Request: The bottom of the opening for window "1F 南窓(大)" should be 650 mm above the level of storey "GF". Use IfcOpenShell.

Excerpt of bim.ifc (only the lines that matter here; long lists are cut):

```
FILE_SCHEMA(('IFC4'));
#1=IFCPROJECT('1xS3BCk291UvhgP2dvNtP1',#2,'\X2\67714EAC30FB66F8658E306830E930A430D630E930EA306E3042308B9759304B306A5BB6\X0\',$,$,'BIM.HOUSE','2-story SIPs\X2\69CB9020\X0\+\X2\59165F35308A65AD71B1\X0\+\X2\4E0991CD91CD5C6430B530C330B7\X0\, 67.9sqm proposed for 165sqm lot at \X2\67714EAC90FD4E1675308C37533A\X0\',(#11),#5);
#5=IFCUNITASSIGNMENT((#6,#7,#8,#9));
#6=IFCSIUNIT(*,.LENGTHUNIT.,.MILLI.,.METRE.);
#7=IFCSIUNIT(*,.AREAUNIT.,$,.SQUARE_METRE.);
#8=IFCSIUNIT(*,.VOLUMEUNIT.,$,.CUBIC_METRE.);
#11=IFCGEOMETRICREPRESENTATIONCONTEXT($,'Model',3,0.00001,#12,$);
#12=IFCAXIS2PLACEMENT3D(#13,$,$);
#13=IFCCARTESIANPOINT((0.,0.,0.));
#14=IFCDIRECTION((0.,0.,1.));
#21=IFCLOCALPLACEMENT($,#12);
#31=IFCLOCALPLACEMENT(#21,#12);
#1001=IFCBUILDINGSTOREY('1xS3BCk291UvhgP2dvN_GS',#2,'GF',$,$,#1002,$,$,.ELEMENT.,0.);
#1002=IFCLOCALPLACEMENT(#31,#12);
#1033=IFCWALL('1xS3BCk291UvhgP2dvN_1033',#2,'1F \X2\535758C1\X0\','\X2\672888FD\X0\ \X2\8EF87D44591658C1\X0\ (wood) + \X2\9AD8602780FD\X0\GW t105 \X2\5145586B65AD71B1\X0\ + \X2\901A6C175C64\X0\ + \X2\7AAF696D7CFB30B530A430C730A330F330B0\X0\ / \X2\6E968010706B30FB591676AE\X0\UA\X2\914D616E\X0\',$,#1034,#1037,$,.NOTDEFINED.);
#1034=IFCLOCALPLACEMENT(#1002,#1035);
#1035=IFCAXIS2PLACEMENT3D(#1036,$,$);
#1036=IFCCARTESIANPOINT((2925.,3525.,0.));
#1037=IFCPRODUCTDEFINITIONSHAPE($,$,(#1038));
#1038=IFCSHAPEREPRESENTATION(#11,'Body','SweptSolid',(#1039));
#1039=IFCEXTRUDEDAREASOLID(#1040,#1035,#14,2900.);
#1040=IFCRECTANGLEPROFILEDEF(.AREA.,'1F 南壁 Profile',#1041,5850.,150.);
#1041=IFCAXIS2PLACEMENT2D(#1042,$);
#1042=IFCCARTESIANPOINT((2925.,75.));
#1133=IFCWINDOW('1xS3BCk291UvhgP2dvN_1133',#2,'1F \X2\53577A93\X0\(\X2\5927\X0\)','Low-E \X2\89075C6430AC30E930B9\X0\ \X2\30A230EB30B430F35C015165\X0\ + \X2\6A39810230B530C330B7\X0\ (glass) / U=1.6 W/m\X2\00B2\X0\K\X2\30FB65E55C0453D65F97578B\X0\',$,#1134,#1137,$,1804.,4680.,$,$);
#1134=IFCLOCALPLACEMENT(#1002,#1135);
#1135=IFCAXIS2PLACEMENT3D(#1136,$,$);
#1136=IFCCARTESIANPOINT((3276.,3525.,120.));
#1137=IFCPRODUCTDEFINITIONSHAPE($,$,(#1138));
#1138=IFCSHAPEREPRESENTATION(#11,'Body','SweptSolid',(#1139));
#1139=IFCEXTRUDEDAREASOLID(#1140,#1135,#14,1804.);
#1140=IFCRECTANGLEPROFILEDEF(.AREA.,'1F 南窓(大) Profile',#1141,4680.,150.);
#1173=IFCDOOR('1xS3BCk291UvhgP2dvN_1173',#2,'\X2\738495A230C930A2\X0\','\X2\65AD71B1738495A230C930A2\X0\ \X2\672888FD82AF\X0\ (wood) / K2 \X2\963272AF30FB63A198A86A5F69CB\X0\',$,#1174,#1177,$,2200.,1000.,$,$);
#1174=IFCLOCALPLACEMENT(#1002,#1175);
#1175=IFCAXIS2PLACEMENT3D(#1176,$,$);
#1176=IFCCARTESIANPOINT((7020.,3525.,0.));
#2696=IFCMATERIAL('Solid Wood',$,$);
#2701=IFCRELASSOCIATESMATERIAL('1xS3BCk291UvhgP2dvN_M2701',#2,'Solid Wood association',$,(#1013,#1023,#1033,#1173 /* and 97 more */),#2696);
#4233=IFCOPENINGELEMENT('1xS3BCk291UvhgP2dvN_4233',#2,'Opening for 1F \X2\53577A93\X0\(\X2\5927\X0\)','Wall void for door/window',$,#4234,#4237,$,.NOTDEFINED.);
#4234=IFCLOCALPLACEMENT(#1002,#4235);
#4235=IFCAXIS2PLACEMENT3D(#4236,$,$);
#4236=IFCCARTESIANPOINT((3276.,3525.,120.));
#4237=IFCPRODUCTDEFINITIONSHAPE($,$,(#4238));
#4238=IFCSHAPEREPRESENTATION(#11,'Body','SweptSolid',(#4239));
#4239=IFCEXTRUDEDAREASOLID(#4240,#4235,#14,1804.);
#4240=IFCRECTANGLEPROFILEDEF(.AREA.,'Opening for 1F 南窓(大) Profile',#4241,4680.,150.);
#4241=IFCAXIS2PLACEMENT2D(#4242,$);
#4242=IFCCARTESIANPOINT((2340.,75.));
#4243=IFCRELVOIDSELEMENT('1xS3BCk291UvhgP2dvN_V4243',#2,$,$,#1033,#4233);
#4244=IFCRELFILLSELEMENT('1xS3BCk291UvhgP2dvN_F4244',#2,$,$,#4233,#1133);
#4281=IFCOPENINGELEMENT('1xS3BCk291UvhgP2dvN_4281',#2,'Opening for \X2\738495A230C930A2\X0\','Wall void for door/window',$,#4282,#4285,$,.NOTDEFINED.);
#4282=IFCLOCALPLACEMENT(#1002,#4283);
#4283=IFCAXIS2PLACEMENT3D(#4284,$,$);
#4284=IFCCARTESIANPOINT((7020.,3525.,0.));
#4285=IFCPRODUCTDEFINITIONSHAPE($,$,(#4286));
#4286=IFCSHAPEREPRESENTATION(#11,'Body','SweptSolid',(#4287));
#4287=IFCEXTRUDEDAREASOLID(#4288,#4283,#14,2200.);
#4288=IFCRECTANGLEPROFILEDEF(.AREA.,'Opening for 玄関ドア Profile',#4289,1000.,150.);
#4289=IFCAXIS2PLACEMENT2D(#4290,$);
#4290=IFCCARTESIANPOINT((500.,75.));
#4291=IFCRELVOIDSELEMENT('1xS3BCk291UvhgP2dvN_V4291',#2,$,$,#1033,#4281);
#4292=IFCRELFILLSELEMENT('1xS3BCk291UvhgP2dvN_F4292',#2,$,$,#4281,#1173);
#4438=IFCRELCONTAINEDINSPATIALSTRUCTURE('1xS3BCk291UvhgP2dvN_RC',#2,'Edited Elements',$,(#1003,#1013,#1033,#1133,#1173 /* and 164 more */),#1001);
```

```python
import numpy as np
import ifcopenshell
import ifcopenshell.api.geometry
import ifcopenshell.geom
import ifcopenshell.util.element
import ifcopenshell.util.placement
import ifcopenshell.util.shape
import ifcopenshell.util.unit

model = ifcopenshell.open("bim.ifc")
unit_scale = ifcopenshell.util.unit.calculate_unit_scale(model)

window = model.by_guid("1xS3BCk291UvhgP2dvN_1133")
opening = window.FillsVoids[0].RelatingOpeningElement
storey = ifcopenshell.util.element.get_container(window, ifc_class="IfcBuildingStorey")
level = ifcopenshell.util.placement.get_local_placement(storey.ObjectPlacement)[2, 3]

# The opening's origin need not be at the sill, so measure its lowest point.
shape = ifcopenshell.geom.create_shape(ifcopenshell.geom.settings(), opening)
bottom = ifcopenshell.util.shape.get_shape_bottom_elevation(shape, shape.geometry) / unit_scale
dz = level + 650.0 - bottom

shift = np.array([0.0, 0.0, dz])
# The window is not placed relative to its opening, so move both.
for product in (opening, window):
    matrix = ifcopenshell.util.placement.get_local_placement(product.ObjectPlacement)
    matrix[:3, 3] += shift
    ifcopenshell.api.geometry.edit_object_placement(model, product=product, matrix=matrix, is_si=False)

print(f"moved by {dz * unit_scale:+.3f} m")

model.write("bim-out.ifc")
```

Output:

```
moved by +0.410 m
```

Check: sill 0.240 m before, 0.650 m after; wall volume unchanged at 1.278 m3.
